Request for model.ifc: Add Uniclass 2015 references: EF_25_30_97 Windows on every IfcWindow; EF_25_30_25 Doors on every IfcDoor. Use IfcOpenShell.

First a look at what the model holds.

```python
import ifcopenshell

model = ifcopenshell.open("model.ifc")
print(model.schema)
print("classifications:", [c.Name for c in model.by_type("IfcClassification")])
for ifc_class in ("IfcDoor", "IfcRoof", "IfcStair", "IfcWall", "IfcWindow"):
    print(ifc_class, len(model.by_type(ifc_class)))
```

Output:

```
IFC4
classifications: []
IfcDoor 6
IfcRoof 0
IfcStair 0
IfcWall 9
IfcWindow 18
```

```python
import ifcopenshell
import ifcopenshell.api.classification

model = ifcopenshell.open("model.ifc")

system = ifcopenshell.api.classification.add_classification(model, classification="Uniclass 2015")

codes = {
    "IfcWindow": ("EF_25_30_97", "Windows"),
    "IfcDoor": ("EF_25_30_25", "Doors"),
}
for ifc_class, (code, name) in codes.items():
    products = model.by_type(ifc_class)
    ifcopenshell.api.classification.add_reference(
        model, products=products, classification=system, identification=code, name=name
    )
    print(code, len(products))

model.write("model_rev.ifc")
```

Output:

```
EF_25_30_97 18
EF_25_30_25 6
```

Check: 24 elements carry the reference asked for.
